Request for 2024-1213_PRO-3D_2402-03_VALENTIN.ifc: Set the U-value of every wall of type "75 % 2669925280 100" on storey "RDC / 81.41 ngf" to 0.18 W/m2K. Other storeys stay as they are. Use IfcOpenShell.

First a look at what the model holds.

```python
import ifcopenshell
import ifcopenshell.util.element

model = ifcopenshell.open("2024-1213_PRO-3D_2402-03_VALENTIN.ifc")
print(model.schema)
storey = next(s for s in model.by_type("IfcBuildingStorey") if s.Name == "RDC / 81.41 ngf")
walls = [e for e in ifcopenshell.util.element.get_decomposition(storey) if e.is_a("IfcWall")]
seen = {}
for e in walls:
    element_type = ifcopenshell.util.element.get_type(e)
    key = (element_type.Name if element_type != e and element_type else None, ifcopenshell.util.element.get_pset(e, "Pset_WallCommon", "ThermalTransmittance"))
    seen[key] = seen.get(key, 0) + 1
for (name, value), count in sorted(seen.items(), key=str):
    print(count, "x", name, "|", value)
```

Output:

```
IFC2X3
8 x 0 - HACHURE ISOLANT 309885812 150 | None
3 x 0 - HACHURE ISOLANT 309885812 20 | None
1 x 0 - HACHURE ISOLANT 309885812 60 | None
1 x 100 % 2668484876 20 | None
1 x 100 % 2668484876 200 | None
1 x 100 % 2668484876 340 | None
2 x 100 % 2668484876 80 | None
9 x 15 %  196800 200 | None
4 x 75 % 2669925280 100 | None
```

```python
import ifcopenshell
import ifcopenshell.api.pset
import ifcopenshell.util.element

model = ifcopenshell.open("2024-1213_PRO-3D_2402-03_VALENTIN.ifc")

storey = next(s for s in model.by_type("IfcBuildingStorey") if s.Name == "RDC / 81.41 ngf")
walls = [e for e in ifcopenshell.util.element.get_decomposition(storey) if e.is_a("IfcWall")]

count = 0
for e in walls:
    element_type = ifcopenshell.util.element.get_type(e)
    if element_type in (None, e) or element_type.Name != "75 % 2669925280 100":
        continue
    # add_pset returns the element's existing set when there is one.
    pset = ifcopenshell.api.pset.add_pset(model, product=e, name="Pset_WallCommon")
    ifcopenshell.api.pset.edit_pset(model, pset=pset, properties={"ThermalTransmittance": 0.18})
    count += 1

print(count, "walls updated")

model.write("2024-1213_PRO-3D_2402-03_VALENTIN_v2.ifc")
```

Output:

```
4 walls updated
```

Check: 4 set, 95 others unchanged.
